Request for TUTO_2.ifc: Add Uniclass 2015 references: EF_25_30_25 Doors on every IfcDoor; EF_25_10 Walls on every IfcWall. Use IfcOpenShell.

First a look at what the model holds.

```python
import ifcopenshell

model = ifcopenshell.open("TUTO_2.ifc")
print(model.schema)
print("classifications:", [c.Name for c in model.by_type("IfcClassification")])
for ifc_class in ("IfcDoor", "IfcRoof", "IfcStair", "IfcWall", "IfcWindow"):
    print(ifc_class, len(model.by_type(ifc_class)))
```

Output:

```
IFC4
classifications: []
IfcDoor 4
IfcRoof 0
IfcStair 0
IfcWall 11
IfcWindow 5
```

```python
import ifcopenshell
import ifcopenshell.api.classification

model = ifcopenshell.open("TUTO_2.ifc")

system = ifcopenshell.api.classification.add_classification(model, classification="Uniclass 2015")

codes = {
    "IfcDoor": ("EF_25_30_25", "Doors"),
    "IfcWall": ("EF_25_10", "Walls"),
}
for ifc_class, (code, name) in codes.items():
    products = model.by_type(ifc_class)
    ifcopenshell.api.classification.add_reference(
        model, products=products, classification=system, identification=code, name=name
    )
    print(code, len(products))

model.write("TUTO_2_rev.ifc")
```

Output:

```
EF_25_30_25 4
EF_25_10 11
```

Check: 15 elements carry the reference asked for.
